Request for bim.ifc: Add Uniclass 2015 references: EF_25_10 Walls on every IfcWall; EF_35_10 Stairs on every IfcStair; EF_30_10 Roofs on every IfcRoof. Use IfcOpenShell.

First a look at what the model holds.

```python
import ifcopenshell

model = ifcopenshell.open("bim.ifc")
print(model.schema)
print("classifications:", [c.Name for c in model.by_type("IfcClassification")])
for ifc_class in ("IfcDoor", "IfcRoof", "IfcStair", "IfcWall", "IfcWindow"):
    print(ifc_class, len(model.by_type(ifc_class)))
```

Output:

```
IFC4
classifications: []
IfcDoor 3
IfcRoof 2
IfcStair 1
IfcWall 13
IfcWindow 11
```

```python
import ifcopenshell
import ifcopenshell.api.classification

model = ifcopenshell.open("bim.ifc")

system = ifcopenshell.api.classification.add_classification(model, classification="Uniclass 2015")

codes = {
    "IfcWall": ("EF_25_10", "Walls"),
    "IfcStair": ("EF_35_10", "Stairs"),
    "IfcRoof": ("EF_30_10", "Roofs"),
}
for ifc_class, (code, name) in codes.items():
    products = model.by_type(ifc_class)
    ifcopenshell.api.classification.add_reference(
        model, products=products, classification=system, identification=code, name=name
    )
    print(code, len(products))

model.write("bim_v2.ifc")
```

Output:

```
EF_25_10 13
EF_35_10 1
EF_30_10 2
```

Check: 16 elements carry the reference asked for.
